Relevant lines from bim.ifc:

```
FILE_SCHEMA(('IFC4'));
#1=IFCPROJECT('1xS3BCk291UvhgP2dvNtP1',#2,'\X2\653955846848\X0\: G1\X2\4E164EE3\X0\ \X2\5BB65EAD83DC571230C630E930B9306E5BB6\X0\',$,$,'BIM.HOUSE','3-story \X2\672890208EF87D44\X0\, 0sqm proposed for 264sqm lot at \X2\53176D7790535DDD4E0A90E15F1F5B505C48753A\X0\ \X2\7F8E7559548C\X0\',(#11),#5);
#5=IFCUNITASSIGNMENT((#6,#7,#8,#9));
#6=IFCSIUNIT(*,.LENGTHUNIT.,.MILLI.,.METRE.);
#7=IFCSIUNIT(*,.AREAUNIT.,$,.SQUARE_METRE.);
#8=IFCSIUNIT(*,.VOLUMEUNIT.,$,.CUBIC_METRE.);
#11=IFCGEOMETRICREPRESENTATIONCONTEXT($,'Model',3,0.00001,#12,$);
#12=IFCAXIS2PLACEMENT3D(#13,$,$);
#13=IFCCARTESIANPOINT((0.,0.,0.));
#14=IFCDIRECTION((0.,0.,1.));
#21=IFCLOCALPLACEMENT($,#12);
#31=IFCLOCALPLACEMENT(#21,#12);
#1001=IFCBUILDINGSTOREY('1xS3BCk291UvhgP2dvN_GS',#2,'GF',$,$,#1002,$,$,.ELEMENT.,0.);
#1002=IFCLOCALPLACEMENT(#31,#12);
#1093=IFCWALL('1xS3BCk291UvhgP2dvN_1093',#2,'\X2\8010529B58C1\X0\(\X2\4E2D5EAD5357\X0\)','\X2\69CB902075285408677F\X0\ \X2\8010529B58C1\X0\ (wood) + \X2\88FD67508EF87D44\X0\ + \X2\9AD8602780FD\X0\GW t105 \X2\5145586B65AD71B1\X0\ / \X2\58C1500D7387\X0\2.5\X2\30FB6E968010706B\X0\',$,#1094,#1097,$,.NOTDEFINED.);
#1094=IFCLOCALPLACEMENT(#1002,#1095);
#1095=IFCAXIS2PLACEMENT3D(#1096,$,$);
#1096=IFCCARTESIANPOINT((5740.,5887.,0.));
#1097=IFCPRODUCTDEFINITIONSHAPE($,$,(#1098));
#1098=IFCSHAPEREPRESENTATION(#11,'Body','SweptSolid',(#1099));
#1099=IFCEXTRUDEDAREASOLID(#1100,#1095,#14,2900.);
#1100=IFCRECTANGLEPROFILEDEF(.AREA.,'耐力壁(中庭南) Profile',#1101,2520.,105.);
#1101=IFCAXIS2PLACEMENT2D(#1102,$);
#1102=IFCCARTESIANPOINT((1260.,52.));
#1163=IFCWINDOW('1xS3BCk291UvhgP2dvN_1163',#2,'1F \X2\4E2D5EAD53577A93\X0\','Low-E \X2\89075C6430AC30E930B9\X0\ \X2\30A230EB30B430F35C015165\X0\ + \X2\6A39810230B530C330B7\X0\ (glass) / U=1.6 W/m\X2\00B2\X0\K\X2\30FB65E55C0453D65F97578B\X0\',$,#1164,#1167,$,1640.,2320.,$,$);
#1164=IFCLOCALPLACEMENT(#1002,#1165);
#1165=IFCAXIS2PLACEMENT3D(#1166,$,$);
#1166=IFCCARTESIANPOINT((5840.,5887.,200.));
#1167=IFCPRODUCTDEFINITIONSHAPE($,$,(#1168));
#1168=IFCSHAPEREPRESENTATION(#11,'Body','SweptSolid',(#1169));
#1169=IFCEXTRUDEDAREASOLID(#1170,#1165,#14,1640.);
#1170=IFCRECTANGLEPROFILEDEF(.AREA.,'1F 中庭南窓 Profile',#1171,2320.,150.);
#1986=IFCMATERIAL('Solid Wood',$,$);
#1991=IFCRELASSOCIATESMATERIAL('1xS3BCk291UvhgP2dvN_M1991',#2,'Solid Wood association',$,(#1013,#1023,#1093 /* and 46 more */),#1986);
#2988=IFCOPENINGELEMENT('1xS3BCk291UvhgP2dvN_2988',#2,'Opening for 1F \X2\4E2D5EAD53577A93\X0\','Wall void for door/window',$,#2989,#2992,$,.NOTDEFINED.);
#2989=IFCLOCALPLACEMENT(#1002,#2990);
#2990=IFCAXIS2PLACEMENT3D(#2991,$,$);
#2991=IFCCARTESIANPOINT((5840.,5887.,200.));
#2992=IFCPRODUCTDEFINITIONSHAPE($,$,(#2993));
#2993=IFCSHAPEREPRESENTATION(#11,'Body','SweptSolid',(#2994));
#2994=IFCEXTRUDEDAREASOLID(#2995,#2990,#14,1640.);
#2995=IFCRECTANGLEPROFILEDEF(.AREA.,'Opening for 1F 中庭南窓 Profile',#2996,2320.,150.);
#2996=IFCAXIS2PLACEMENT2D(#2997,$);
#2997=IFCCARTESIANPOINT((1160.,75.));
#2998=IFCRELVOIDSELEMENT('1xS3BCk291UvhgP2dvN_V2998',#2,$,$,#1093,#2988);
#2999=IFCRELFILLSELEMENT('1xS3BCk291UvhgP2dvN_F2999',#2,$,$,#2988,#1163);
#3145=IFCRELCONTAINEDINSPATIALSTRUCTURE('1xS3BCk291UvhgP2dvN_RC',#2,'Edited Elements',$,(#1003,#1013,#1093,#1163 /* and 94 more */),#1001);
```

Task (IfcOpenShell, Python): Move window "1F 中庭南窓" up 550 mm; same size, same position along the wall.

```python
import numpy as np
import ifcopenshell
import ifcopenshell.api.geometry
import ifcopenshell.util.placement
import ifcopenshell.util.unit

model = ifcopenshell.open("bim.ifc")
unit_scale = ifcopenshell.util.unit.calculate_unit_scale(model)

window = model.by_id(1163)
opening = window.FillsVoids[0].RelatingOpeningElement
dz = 0.55 / unit_scale

shift = np.array([0.0, 0.0, dz])
# The window is not placed relative to its opening, so move both.
for product in (opening, window):
    matrix = ifcopenshell.util.placement.get_local_placement(product.ObjectPlacement)
    matrix[:3, 3] += shift
    ifcopenshell.api.geometry.edit_object_placement(model, product=product, matrix=matrix, is_si=False)

print(f"moved by {dz * unit_scale:+.3f} m")

model.write("bim_edited.ifc")
```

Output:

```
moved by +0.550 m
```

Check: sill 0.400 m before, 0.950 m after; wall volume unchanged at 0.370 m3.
